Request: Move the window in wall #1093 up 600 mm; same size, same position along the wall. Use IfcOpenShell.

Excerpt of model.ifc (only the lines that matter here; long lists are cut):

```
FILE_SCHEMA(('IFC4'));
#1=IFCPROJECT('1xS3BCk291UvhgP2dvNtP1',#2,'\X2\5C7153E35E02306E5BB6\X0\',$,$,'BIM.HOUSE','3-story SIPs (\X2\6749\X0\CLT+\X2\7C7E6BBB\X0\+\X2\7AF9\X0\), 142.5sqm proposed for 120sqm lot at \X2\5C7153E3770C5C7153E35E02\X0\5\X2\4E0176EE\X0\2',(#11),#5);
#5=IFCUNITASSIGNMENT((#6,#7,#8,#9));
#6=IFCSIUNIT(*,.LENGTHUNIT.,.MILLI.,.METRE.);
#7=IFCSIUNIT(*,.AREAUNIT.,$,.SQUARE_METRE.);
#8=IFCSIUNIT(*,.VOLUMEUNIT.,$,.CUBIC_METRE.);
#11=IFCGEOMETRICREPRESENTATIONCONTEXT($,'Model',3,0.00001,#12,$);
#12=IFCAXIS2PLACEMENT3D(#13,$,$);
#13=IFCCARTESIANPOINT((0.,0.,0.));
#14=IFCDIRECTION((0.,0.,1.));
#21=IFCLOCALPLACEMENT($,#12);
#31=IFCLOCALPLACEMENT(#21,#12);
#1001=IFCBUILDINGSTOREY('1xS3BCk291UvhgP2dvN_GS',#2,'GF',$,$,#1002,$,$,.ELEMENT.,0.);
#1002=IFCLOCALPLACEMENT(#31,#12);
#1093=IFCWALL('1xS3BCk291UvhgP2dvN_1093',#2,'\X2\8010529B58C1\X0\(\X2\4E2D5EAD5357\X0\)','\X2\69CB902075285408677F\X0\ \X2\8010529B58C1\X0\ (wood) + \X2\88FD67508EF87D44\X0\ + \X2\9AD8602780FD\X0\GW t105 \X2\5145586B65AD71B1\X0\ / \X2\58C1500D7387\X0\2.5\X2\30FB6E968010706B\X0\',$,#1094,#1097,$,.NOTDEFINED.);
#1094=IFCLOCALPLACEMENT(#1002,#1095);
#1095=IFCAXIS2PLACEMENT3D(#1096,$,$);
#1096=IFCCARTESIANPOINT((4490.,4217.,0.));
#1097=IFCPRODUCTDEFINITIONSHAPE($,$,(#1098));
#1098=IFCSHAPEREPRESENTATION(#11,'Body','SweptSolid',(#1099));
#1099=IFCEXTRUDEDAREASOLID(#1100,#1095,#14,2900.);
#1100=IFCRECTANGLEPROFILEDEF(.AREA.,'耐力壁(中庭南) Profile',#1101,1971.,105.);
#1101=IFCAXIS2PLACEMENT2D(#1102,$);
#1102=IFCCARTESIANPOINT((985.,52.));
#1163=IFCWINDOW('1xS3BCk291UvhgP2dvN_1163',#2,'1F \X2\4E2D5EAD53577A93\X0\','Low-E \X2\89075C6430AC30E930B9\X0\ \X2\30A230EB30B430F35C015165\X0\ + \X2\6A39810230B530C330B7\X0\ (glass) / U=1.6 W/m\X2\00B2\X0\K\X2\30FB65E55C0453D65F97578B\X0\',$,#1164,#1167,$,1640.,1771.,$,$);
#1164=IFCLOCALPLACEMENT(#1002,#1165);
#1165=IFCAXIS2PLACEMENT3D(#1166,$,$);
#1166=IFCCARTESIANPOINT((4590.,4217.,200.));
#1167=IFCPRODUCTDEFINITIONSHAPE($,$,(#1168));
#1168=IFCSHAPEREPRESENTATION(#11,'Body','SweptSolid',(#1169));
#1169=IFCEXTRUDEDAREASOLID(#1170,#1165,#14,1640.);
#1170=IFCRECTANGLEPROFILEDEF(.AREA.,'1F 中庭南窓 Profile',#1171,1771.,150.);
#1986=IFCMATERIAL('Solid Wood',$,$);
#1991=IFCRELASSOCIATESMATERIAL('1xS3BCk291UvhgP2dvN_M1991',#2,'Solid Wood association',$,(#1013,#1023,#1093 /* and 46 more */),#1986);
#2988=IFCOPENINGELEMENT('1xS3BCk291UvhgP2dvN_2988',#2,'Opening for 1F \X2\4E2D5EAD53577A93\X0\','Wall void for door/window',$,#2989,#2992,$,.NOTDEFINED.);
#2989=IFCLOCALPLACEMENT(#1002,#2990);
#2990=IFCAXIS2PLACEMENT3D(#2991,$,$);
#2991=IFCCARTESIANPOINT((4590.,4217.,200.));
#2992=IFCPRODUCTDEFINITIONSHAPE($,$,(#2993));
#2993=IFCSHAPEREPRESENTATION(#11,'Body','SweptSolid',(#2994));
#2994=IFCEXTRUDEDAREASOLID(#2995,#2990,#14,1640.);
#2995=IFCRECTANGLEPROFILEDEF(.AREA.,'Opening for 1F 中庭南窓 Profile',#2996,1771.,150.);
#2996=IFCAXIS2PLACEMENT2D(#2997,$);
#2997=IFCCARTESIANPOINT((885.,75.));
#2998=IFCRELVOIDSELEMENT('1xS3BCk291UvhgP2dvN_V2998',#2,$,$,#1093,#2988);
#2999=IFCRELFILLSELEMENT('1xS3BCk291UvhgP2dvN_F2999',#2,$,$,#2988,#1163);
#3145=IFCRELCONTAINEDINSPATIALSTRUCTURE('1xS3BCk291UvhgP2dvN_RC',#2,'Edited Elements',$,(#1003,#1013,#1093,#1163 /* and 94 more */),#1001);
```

```python
import numpy as np
import ifcopenshell
import ifcopenshell.api.geometry
import ifcopenshell.util.placement
import ifcopenshell.util.unit

model = ifcopenshell.open("model.ifc")
unit_scale = ifcopenshell.util.unit.calculate_unit_scale(model)

window = model.by_guid("1xS3BCk291UvhgP2dvN_1163")
opening = window.FillsVoids[0].RelatingOpeningElement
dz = 0.6 / unit_scale

shift = np.array([0.0, 0.0, dz])
# The window is not placed relative to its opening, so move both.
for product in (opening, window):
    matrix = ifcopenshell.util.placement.get_local_placement(product.ObjectPlacement)
    matrix[:3, 3] += shift
    ifcopenshell.api.geometry.edit_object_placement(model, product=product, matrix=matrix, is_si=False)

print(f"moved by {dz * unit_scale:+.3f} m")

model.write("model_v2.ifc")
```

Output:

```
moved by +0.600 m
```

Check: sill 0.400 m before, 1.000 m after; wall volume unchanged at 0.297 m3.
